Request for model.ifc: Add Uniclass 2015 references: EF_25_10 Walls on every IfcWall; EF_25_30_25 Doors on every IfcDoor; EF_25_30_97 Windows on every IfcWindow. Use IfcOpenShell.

First a look at what the model holds.

```python
import ifcopenshell

model = ifcopenshell.open("model.ifc")
print(model.schema)
print("classifications:", [c.Name for c in model.by_type("IfcClassification")])
for ifc_class in ("IfcDoor", "IfcRoof", "IfcStair", "IfcWall", "IfcWindow"):
    print(ifc_class, len(model.by_type(ifc_class)))
```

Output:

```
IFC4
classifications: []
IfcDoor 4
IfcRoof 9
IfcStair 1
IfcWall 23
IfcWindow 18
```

```python
import ifcopenshell
import ifcopenshell.api.classification

model = ifcopenshell.open("model.ifc")

system = ifcopenshell.api.classification.add_classification(model, classification="Uniclass 2015")

codes = {
    "IfcWall": ("EF_25_10", "Walls"),
    "IfcDoor": ("EF_25_30_25", "Doors"),
    "IfcWindow": ("EF_25_30_97", "Windows"),
}
for ifc_class, (code, name) in codes.items():
    products = model.by_type(ifc_class)
    ifcopenshell.api.classification.add_reference(
        model, products=products, classification=system, identification=code, name=name
    )
    print(code, len(products))

model.write("model_rev.ifc")
```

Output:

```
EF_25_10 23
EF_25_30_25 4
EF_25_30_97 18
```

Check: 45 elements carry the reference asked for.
